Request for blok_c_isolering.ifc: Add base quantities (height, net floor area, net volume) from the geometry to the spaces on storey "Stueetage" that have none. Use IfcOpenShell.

First a look at what the model holds.

```python
import ifcopenshell
import ifcopenshell.util.element
import ifcopenshell.util.unit

model = ifcopenshell.open("blok_c_isolering.ifc")
print(model.schema)
for unit_type in ("LENGTHUNIT", "AREAUNIT", "VOLUMEUNIT"):
    print(unit_type, ifcopenshell.util.unit.calculate_unit_scale(model, unit_type))
storey = next(s for s in model.by_type("IfcBuildingStorey") if s.Name == "Stueetage")
spaces = [e for e in ifcopenshell.util.element.get_decomposition(storey) if e.is_a("IfcSpace")]
for e in sorted(spaces, key=lambda e: e.id()):
    print(e.id(), e.is_a(), e.Name, list(ifcopenshell.util.element.get_psets(e, qtos_only=True)), sep=" | ")
```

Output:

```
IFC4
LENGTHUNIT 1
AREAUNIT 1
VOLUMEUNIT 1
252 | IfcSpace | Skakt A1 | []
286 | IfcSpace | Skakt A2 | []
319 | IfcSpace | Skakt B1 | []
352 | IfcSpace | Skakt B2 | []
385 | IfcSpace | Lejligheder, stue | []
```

```python
import ifcopenshell
import ifcopenshell.api.pset
import ifcopenshell.geom
import ifcopenshell.util.element
import ifcopenshell.util.shape
import ifcopenshell.util.unit

model = ifcopenshell.open("blok_c_isolering.ifc")
unit_scale = ifcopenshell.util.unit.calculate_unit_scale(model)
area_scale = ifcopenshell.util.unit.calculate_unit_scale(model, "AREAUNIT")
volume_scale = ifcopenshell.util.unit.calculate_unit_scale(model, "VOLUMEUNIT")
settings = ifcopenshell.geom.settings()

storey = next(s for s in model.by_type("IfcBuildingStorey") if s.Name == "Stueetage")
spaces = [e for e in ifcopenshell.util.element.get_decomposition(storey) if e.is_a("IfcSpace")]

for e in sorted(spaces, key=lambda e: e.id()):
    if ifcopenshell.util.element.get_psets(e, qtos_only=True, should_inherit=False):
        continue
    # Geometry comes back in metres, in the element's own axes.
    shape = ifcopenshell.geom.create_shape(settings, e)
    values = {
        "Height": ifcopenshell.util.shape.get_z(shape.geometry) / unit_scale,
        "NetFloorArea": ifcopenshell.util.shape.get_footprint_area(shape.geometry) / area_scale,
        "NetVolume": ifcopenshell.util.shape.get_volume(shape.geometry) / volume_scale,
    }
    qto = ifcopenshell.api.pset.add_qto(model, product=e, name="Qto_SpaceBaseQuantities")
    ifcopenshell.api.pset.edit_qto(model, qto=qto, properties=values)
    print(e.id(), {k: round(v, 3) for k, v in values.items()})

model.write("blok_c_isolering_edited.ifc")
```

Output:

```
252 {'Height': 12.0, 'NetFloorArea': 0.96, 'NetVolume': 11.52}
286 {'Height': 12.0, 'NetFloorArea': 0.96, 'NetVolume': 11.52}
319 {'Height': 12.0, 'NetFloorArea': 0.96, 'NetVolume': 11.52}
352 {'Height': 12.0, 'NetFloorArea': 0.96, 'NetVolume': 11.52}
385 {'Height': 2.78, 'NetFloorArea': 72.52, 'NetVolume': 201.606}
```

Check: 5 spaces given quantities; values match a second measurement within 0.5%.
